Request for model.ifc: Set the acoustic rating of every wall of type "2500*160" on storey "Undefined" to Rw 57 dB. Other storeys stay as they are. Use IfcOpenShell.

First a look at what the model holds.

```python
import ifcopenshell
import ifcopenshell.util.element

model = ifcopenshell.open("model.ifc")
print(model.schema)
storey = next(s for s in model.by_type("IfcBuildingStorey") if s.Name == "Undefined")
walls = [e for e in ifcopenshell.util.element.get_decomposition(storey) if e.is_a("IfcWall")]
seen = {}
for e in walls:
    element_type = ifcopenshell.util.element.get_type(e)
    key = (element_type.Name if element_type != e and element_type else None, ifcopenshell.util.element.get_pset(e, "Pset_WallCommon", "AcousticRating"))
    seen[key] = seen.get(key, 0) + 1
for (name, value), count in sorted(seen.items(), key=str):
    print(count, "x", name, "|", value)
```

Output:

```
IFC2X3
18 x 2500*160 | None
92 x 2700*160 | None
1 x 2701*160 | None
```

```python
import ifcopenshell
import ifcopenshell.api.pset
import ifcopenshell.util.element

model = ifcopenshell.open("model.ifc")

storey = next(s for s in model.by_type("IfcBuildingStorey") if s.Name == "Undefined")
walls = [e for e in ifcopenshell.util.element.get_decomposition(storey) if e.is_a("IfcWall")]

count = 0
for e in walls:
    element_type = ifcopenshell.util.element.get_type(e)
    if element_type in (None, e) or element_type.Name != "2500*160":
        continue
    # add_pset returns the element's existing set when there is one.
    pset = ifcopenshell.api.pset.add_pset(model, product=e, name="Pset_WallCommon")
    ifcopenshell.api.pset.edit_pset(model, pset=pset, properties={"AcousticRating": "Rw 57 dB"})
    count += 1

print(count, "walls updated")

model.write("model_v2.ifc")
```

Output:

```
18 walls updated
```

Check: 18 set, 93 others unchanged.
